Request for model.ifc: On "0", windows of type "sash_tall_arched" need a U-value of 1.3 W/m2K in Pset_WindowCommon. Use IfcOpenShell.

First a look at what the model holds.

```python
import ifcopenshell
import ifcopenshell.util.element

model = ifcopenshell.open("model.ifc")
print(model.schema)
storey = next(s for s in model.by_type("IfcBuildingStorey") if s.Name == "0")
windows = [e for e in ifcopenshell.util.element.get_decomposition(storey) if e.is_a("IfcWindow")]
seen = {}
for e in windows:
    element_type = ifcopenshell.util.element.get_type(e)
    key = (element_type.Name if element_type != e and element_type else None, ifcopenshell.util.element.get_pset(e, "Pset_WindowCommon", "ThermalTransmittance"))
    seen[key] = seen.get(key, 0) + 1
for (name, value), count in sorted(seen.items(), key=str):
    print(count, "x", name, "|", value)
```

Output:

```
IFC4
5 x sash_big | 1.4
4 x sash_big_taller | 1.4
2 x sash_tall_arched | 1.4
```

```python
import ifcopenshell
import ifcopenshell.api.pset
import ifcopenshell.util.element

model = ifcopenshell.open("model.ifc")

storey = next(s for s in model.by_type("IfcBuildingStorey") if s.Name == "0")
windows = [e for e in ifcopenshell.util.element.get_decomposition(storey) if e.is_a("IfcWindow")]

count = 0
for e in windows:
    element_type = ifcopenshell.util.element.get_type(e)
    if element_type in (None, e) or element_type.Name != "sash_tall_arched":
        continue
    # add_pset returns the element's existing set when there is one.
    pset = ifcopenshell.api.pset.add_pset(model, product=e, name="Pset_WindowCommon")
    ifcopenshell.api.pset.edit_pset(model, pset=pset, properties={"ThermalTransmittance": 1.3})
    count += 1

print(count, "windows updated")

model.write("model_updated.ifc")
```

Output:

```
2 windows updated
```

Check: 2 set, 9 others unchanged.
